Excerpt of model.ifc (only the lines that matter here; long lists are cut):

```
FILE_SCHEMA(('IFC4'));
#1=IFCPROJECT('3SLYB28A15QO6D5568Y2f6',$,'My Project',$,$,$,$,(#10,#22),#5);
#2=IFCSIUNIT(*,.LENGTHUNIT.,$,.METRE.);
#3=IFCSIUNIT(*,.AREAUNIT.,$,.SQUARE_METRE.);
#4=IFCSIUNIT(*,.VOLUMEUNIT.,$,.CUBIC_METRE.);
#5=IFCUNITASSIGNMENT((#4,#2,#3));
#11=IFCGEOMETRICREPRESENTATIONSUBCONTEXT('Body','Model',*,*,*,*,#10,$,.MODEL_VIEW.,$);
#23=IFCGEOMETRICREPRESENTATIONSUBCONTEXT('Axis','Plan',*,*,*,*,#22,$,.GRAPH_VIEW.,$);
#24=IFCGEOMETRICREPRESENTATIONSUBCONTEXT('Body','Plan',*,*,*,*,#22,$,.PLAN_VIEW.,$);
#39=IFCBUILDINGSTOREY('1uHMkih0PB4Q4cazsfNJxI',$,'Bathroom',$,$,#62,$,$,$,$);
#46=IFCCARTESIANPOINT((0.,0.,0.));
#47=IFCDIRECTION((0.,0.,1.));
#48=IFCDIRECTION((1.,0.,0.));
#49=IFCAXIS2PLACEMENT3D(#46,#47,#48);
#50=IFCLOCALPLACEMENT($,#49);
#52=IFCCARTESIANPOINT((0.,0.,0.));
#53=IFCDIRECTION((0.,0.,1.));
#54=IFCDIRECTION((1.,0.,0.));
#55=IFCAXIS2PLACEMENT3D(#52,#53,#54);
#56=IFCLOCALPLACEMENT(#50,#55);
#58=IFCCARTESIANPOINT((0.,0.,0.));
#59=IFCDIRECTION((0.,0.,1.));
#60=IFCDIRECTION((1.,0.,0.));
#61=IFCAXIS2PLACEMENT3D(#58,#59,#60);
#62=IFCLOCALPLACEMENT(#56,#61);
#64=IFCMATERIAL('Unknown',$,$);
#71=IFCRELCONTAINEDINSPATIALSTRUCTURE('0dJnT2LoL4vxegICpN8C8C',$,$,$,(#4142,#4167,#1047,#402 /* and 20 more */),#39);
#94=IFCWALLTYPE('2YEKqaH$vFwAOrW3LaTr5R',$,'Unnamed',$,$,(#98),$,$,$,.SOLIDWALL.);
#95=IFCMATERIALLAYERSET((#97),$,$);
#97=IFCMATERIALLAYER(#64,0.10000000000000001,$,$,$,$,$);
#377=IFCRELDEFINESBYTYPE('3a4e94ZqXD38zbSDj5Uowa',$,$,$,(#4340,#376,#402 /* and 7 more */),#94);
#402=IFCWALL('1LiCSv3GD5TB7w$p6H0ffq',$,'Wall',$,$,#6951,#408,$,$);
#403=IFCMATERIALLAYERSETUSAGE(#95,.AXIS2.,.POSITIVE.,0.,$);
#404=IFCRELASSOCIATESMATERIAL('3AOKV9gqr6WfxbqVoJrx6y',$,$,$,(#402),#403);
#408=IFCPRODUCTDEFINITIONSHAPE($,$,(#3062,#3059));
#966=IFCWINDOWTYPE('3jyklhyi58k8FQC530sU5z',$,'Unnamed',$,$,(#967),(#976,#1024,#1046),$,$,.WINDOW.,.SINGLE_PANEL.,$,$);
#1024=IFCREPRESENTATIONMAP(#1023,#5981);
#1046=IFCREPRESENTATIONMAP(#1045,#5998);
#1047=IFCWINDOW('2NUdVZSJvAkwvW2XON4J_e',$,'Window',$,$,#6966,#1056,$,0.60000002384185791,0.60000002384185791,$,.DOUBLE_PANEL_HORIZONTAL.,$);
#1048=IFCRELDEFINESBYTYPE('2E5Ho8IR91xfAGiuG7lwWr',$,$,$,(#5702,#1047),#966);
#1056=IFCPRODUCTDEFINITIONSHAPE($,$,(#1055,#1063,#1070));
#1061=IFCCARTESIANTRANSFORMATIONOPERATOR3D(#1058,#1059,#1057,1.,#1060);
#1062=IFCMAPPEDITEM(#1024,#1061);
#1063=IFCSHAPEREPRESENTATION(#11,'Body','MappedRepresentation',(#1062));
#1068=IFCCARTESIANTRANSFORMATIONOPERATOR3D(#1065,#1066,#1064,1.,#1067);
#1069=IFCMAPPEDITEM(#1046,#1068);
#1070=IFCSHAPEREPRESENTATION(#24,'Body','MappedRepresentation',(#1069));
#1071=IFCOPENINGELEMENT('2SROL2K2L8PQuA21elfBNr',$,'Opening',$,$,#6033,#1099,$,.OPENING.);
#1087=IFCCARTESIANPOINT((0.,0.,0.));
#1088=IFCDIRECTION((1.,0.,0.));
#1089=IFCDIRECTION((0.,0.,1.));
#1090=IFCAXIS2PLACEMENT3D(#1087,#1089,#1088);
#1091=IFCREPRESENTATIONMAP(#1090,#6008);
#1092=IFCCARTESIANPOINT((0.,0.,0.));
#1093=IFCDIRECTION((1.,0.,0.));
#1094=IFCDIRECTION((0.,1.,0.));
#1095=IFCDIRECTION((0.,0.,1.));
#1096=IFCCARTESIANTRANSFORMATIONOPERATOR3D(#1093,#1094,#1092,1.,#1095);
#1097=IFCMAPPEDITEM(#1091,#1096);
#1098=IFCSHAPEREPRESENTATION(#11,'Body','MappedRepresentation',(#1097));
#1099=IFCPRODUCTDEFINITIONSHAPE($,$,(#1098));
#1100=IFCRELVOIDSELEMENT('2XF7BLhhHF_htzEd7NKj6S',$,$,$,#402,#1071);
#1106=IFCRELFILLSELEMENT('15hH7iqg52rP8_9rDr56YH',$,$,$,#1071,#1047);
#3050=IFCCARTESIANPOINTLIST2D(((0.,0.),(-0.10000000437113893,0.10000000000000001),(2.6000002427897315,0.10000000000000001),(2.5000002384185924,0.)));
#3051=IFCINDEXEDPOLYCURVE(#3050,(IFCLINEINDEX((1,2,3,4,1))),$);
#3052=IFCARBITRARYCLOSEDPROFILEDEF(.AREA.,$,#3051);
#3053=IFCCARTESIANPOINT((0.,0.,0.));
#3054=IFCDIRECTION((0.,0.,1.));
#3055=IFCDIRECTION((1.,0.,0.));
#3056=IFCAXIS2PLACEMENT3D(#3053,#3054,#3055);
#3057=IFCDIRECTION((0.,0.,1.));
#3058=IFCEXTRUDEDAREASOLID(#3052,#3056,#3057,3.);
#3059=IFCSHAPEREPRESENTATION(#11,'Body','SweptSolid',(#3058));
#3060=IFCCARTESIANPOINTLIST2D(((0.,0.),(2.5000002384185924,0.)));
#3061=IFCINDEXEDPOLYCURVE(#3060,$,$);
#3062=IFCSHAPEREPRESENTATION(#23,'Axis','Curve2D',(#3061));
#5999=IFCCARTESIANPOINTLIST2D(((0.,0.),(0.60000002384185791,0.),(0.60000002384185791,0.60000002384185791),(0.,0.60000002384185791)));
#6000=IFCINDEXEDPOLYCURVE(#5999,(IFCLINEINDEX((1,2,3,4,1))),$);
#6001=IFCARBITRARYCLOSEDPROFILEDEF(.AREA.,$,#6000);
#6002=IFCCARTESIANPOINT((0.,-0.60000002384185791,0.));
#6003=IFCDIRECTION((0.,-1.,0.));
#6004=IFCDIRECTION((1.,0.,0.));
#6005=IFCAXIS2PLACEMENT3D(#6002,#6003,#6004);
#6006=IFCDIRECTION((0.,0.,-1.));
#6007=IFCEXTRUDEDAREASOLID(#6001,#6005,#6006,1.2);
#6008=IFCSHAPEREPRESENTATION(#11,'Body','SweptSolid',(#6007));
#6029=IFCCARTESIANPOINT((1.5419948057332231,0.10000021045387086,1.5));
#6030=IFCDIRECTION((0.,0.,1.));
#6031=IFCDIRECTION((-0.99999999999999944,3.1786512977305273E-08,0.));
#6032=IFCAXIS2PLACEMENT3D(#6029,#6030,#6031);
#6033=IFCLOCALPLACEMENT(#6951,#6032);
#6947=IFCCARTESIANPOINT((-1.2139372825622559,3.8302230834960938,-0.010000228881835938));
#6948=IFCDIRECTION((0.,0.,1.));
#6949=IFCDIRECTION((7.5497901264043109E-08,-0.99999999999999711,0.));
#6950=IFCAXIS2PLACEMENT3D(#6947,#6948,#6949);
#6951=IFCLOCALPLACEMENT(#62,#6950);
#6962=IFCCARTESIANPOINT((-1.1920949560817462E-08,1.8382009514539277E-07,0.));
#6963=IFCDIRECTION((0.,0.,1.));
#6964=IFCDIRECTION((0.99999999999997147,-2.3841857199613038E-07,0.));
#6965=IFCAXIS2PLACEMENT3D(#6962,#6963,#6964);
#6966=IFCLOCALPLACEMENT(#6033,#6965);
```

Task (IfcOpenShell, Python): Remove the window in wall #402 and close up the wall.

```python
import ifcopenshell
import ifcopenshell.api.feature
import ifcopenshell.api.root
import ifcopenshell.geom
import ifcopenshell.util.shape

model = ifcopenshell.open("model.ifc")
settings = ifcopenshell.geom.settings()


def volume(element):
    """Net volume in cubic metres, openings subtracted."""
    shape = ifcopenshell.geom.create_shape(settings, element)
    return ifcopenshell.util.shape.get_volume(shape.geometry)


window = model.by_id(1047)
opening = window.FillsVoids[0].RelatingOpeningElement
wall = opening.VoidsElements[0].RelatingBuildingElement
before = volume(wall)

ifcopenshell.api.root.remove_product(model, product=window)
ifcopenshell.api.feature.remove_feature(model, feature=opening)

after = volume(wall)

print(f"wall volume {before:.3f} -> {after:.3f} m3")

model.write("model-out.ifc")
```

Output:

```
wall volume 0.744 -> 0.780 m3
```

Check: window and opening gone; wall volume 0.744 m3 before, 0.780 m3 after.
